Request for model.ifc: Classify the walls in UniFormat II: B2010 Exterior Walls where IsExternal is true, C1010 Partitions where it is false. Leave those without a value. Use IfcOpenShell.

First a look at what the model holds.

```python
import ifcopenshell
import ifcopenshell.util.element

model = ifcopenshell.open("model.ifc")
print(model.schema)
print("classifications:", [c.Name for c in model.by_type("IfcClassification")])
values = [ifcopenshell.util.element.get_pset(e, "Pset_WallCommon", "IsExternal") for e in model.by_type("IfcWall")]
for value in (True, False, None):
    print("IsExternal", value, values.count(value))
```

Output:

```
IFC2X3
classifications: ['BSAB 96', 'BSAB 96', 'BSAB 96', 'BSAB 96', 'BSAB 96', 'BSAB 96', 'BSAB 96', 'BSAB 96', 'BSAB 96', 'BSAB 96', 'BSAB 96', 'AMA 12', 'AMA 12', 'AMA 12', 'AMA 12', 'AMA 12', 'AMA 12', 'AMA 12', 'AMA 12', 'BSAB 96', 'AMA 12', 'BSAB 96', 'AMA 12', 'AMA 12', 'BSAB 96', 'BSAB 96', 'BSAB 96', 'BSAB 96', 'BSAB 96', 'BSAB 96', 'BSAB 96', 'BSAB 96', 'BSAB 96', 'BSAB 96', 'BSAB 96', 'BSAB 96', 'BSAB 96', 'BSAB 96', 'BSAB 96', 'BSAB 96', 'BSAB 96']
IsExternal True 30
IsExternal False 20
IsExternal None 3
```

```python
import ifcopenshell
import ifcopenshell.api.classification
import ifcopenshell.util.element

model = ifcopenshell.open("model.ifc")

# IFC2X3 requires Source and Edition and has no link from the project to the system.
system = model.create_entity("IfcClassification", Source="ASTM", Edition="E1557", Name="UniFormat II")

walls = model.by_type("IfcWall")
external = {e: ifcopenshell.util.element.get_pset(e, "Pset_WallCommon", "IsExternal") for e in walls}
for flag, code, name in ((True, "B2010", "Exterior Walls"), (False, "C1010", "Partitions")):
    products = [e for e in walls if external[e] is flag]
    ifcopenshell.api.classification.add_reference(
        model, products=products, classification=system, identification=code, name=name
    )
    print(code, len(products))

model.write("model_edited.ifc")
```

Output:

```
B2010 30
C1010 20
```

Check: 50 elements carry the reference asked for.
